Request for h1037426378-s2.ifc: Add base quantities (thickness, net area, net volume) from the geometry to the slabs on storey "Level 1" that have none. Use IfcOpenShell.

First a look at what the model holds.

```python
import ifcopenshell
import ifcopenshell.util.element
import ifcopenshell.util.unit

model = ifcopenshell.open("h1037426378-s2.ifc")
print(model.schema)
for unit_type in ("LENGTHUNIT", "AREAUNIT", "VOLUMEUNIT"):
    print(unit_type, ifcopenshell.util.unit.calculate_unit_scale(model, unit_type))
storey = next(s for s in model.by_type("IfcBuildingStorey") if s.Name == "Level 1")
slabs = [e for e in ifcopenshell.util.element.get_decomposition(storey) if e.is_a("IfcSlab")]
for e in sorted(slabs, key=lambda e: e.id()):
    print(e.id(), e.is_a(), e.Name, list(ifcopenshell.util.element.get_psets(e, qtos_only=True)), sep=" | ")
```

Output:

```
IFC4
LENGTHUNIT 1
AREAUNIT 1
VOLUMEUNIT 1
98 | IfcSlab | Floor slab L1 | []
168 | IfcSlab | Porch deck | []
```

```python
import ifcopenshell
import ifcopenshell.api.pset
import ifcopenshell.geom
import ifcopenshell.util.element
import ifcopenshell.util.shape
import ifcopenshell.util.unit

model = ifcopenshell.open("h1037426378-s2.ifc")
unit_scale = ifcopenshell.util.unit.calculate_unit_scale(model)
area_scale = ifcopenshell.util.unit.calculate_unit_scale(model, "AREAUNIT")
volume_scale = ifcopenshell.util.unit.calculate_unit_scale(model, "VOLUMEUNIT")
settings = ifcopenshell.geom.settings()

storey = next(s for s in model.by_type("IfcBuildingStorey") if s.Name == "Level 1")
slabs = [e for e in ifcopenshell.util.element.get_decomposition(storey) if e.is_a("IfcSlab")]

for e in sorted(slabs, key=lambda e: e.id()):
    if ifcopenshell.util.element.get_psets(e, qtos_only=True, should_inherit=False):
        continue
    # Geometry comes back in metres, in the element's own axes.
    shape = ifcopenshell.geom.create_shape(settings, e)
    values = {
        "Width": ifcopenshell.util.shape.get_z(shape.geometry) / unit_scale,
        "NetArea": ifcopenshell.util.shape.get_footprint_area(shape.geometry) / area_scale,
        "NetVolume": ifcopenshell.util.shape.get_volume(shape.geometry) / volume_scale,
    }
    qto = ifcopenshell.api.pset.add_qto(model, product=e, name="Qto_SlabBaseQuantities")
    ifcopenshell.api.pset.edit_qto(model, qto=qto, properties=values)
    print(e.id(), {k: round(v, 3) for k, v in values.items()})

model.write("h1037426378-s2_v2.ifc")
```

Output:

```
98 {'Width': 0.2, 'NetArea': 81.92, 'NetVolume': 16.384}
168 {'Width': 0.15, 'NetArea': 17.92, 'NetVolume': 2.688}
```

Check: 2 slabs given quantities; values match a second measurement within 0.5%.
